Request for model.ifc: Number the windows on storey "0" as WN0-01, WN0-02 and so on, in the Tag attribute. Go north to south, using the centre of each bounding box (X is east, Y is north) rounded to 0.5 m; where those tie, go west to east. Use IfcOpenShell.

First a look at what the model holds.

```python
import ifcopenshell
import ifcopenshell.util.element
import ifcopenshell.util.placement

model = ifcopenshell.open("model.ifc")
print(model.schema)
storey = next(s for s in model.by_type("IfcBuildingStorey") if s.Name == "0")
windows = [e for e in ifcopenshell.util.element.get_decomposition(storey) if e.is_a("IfcWindow")]
for e in sorted(windows, key=lambda e: e.id()):
    origin = ifcopenshell.util.placement.get_local_placement(e.ObjectPlacement)[:3, 3]
    print(e.id(), e.Tag, e.Name, origin.round(2) + 0.0, sep=" | ")
```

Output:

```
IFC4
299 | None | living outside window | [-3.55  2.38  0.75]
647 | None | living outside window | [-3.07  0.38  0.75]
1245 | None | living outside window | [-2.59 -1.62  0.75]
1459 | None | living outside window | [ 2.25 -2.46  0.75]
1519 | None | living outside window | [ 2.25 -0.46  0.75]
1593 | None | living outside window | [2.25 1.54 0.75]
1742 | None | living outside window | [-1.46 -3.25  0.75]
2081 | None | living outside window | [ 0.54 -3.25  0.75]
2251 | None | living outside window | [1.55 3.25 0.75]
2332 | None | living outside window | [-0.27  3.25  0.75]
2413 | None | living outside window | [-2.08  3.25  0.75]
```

```python
import ifcopenshell
import ifcopenshell.geom
import ifcopenshell.util.element
import ifcopenshell.util.shape

model = ifcopenshell.open("model.ifc")
settings = ifcopenshell.geom.settings()
settings.set("use-world-coords", True)


def centre(element):
    shape = ifcopenshell.geom.create_shape(settings, element)
    return ifcopenshell.util.shape.get_bbox_centroid(shape.geometry)


storey = next(s for s in model.by_type("IfcBuildingStorey") if s.Name == "0")
windows = [e for e in ifcopenshell.util.element.get_decomposition(storey) if e.is_a("IfcWindow")]

# Insertion points can sit at a corner or the storey origin, so sort by the geometry (in metres).
centres = {e: centre(e) for e in windows}
windows.sort(key=lambda e: (-round(centres[e][1] / 0.5), centres[e][0]))

for i, e in enumerate(windows, start=1):
    number = f"WN0-{i:02d}"
    e.Tag = number
    print(e.id(), number)

model.write("model_updated.ifc")
```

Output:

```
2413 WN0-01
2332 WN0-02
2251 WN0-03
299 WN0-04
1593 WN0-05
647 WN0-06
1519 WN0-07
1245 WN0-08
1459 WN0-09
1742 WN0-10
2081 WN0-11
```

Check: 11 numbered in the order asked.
